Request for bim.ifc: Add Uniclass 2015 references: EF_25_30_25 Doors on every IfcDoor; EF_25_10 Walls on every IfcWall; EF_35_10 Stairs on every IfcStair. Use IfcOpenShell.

First a look at what the model holds.

```python
import ifcopenshell

model = ifcopenshell.open("bim.ifc")
print(model.schema)
print("classifications:", [c.Name for c in model.by_type("IfcClassification")])
for ifc_class in ("IfcDoor", "IfcRoof", "IfcStair", "IfcWall", "IfcWindow"):
    print(ifc_class, len(model.by_type(ifc_class)))
```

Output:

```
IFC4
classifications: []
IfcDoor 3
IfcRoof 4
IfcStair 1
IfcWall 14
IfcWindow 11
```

```python
import ifcopenshell
import ifcopenshell.api.classification

model = ifcopenshell.open("bim.ifc")

system = ifcopenshell.api.classification.add_classification(model, classification="Uniclass 2015")

codes = {
    "IfcDoor": ("EF_25_30_25", "Doors"),
    "IfcWall": ("EF_25_10", "Walls"),
    "IfcStair": ("EF_35_10", "Stairs"),
}
for ifc_class, (code, name) in codes.items():
    products = model.by_type(ifc_class)
    ifcopenshell.api.classification.add_reference(
        model, products=products, classification=system, identification=code, name=name
    )
    print(code, len(products))

model.write("bim_v2.ifc")
```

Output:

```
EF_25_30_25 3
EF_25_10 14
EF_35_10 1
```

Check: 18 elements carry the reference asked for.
